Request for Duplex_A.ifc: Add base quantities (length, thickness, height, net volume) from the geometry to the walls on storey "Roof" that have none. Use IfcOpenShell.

First a look at what the model holds.

```python
import ifcopenshell
import ifcopenshell.util.element
import ifcopenshell.util.unit

model = ifcopenshell.open("Duplex_A.ifc")
print(model.schema)
for unit_type in ("LENGTHUNIT", "AREAUNIT", "VOLUMEUNIT"):
    print(unit_type, ifcopenshell.util.unit.calculate_unit_scale(model, unit_type))
storey = next(s for s in model.by_type("IfcBuildingStorey") if s.Name == "Roof")
walls = [e for e in ifcopenshell.util.element.get_decomposition(storey) if e.is_a("IfcWall")]
for e in sorted(walls, key=lambda e: e.id()):
    print(e.id(), e.is_a(), e.Name, list(ifcopenshell.util.element.get_psets(e, qtos_only=True)), sep=" | ")
```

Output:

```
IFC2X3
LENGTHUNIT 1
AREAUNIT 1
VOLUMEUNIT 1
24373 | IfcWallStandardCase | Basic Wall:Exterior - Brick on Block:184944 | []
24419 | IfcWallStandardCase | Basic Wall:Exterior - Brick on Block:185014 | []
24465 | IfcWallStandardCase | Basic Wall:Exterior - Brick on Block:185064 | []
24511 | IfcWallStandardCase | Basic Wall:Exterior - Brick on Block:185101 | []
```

```python
import ifcopenshell
import ifcopenshell.api.pset
import ifcopenshell.geom
import ifcopenshell.util.element
import ifcopenshell.util.shape
import ifcopenshell.util.unit

model = ifcopenshell.open("Duplex_A.ifc")
unit_scale = ifcopenshell.util.unit.calculate_unit_scale(model)
volume_scale = ifcopenshell.util.unit.calculate_unit_scale(model, "VOLUMEUNIT")
settings = ifcopenshell.geom.settings()

storey = next(s for s in model.by_type("IfcBuildingStorey") if s.Name == "Roof")
walls = [e for e in ifcopenshell.util.element.get_decomposition(storey) if e.is_a("IfcWall")]

for e in sorted(walls, key=lambda e: e.id()):
    if ifcopenshell.util.element.get_psets(e, qtos_only=True, should_inherit=False):
        continue
    # Geometry comes back in metres, in the element's own axes.
    shape = ifcopenshell.geom.create_shape(settings, e)
    values = {
        "Length": ifcopenshell.util.shape.get_x(shape.geometry) / unit_scale,
        "Width": ifcopenshell.util.shape.get_y(shape.geometry) / unit_scale,
        "Height": ifcopenshell.util.shape.get_z(shape.geometry) / unit_scale,
        "NetVolume": ifcopenshell.util.shape.get_volume(shape.geometry) / volume_scale,
    }
    qto = ifcopenshell.api.pset.add_qto(model, product=e, name="BaseQuantities")
    ifcopenshell.api.pset.edit_qto(model, qto=qto, properties=values)
    print(e.id(), {k: round(v, 3) for k, v in values.items()})

model.write("Duplex_A-out.ifc")
```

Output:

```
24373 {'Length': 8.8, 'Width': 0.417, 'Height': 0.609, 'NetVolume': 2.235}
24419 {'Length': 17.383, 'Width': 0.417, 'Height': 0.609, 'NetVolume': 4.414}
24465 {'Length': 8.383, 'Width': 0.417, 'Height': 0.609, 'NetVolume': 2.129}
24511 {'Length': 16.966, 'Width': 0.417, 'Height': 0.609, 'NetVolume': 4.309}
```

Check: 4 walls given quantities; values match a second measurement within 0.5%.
